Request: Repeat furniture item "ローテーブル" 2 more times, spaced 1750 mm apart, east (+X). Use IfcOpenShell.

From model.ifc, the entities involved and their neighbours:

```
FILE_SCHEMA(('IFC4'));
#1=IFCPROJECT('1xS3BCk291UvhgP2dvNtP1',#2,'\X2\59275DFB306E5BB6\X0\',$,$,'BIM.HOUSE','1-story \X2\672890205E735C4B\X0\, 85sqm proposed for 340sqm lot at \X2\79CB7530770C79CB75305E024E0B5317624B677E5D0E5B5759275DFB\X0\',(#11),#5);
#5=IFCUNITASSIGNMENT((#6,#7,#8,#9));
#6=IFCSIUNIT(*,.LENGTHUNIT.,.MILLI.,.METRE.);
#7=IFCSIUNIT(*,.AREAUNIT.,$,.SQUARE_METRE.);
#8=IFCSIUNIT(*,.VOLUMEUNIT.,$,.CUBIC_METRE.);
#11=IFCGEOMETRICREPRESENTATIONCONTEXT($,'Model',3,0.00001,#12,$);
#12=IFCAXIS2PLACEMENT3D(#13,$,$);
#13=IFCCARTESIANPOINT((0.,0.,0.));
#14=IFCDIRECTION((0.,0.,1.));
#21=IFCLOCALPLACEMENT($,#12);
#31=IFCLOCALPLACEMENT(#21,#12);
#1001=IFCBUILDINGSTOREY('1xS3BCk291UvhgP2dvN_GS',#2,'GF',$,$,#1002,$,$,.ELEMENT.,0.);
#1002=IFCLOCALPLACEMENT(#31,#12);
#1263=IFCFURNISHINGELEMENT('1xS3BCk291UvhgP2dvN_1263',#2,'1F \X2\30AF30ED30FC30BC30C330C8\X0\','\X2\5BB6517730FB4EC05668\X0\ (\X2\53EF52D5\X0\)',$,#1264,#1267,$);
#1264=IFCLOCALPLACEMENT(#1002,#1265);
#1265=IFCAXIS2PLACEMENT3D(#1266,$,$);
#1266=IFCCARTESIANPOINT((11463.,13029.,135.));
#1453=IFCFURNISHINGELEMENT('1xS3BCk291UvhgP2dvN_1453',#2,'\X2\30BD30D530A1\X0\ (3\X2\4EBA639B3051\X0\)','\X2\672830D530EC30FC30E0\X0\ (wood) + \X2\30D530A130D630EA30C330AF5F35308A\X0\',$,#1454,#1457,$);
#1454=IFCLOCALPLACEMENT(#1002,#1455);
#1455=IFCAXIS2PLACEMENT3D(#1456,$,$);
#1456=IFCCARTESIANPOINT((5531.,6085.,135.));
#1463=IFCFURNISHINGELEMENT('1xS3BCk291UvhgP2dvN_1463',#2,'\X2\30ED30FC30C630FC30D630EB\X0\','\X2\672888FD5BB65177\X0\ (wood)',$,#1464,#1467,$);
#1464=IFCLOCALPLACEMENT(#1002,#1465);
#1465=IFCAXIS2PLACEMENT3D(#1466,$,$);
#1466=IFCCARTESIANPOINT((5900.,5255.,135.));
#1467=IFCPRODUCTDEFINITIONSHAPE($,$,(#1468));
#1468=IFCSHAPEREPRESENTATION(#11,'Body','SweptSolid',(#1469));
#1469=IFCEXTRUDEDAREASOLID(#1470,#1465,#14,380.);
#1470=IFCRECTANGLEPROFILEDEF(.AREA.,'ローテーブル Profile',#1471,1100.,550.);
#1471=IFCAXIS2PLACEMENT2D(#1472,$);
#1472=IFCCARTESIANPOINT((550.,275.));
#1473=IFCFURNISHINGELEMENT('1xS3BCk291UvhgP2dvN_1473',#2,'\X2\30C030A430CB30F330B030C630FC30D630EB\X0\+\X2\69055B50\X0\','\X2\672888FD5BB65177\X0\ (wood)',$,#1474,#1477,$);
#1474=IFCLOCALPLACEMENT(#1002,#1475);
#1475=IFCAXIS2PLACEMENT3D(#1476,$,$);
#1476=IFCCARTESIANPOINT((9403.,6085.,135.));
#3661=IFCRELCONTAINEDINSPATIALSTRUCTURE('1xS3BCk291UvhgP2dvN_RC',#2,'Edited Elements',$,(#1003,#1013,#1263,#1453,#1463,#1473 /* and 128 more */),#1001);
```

```python
import numpy as np
import ifcopenshell
import ifcopenshell.api.geometry
import ifcopenshell.api.root
import ifcopenshell.util.element
import ifcopenshell.util.placement
import ifcopenshell.util.unit

model = ifcopenshell.open("model.ifc")
unit_scale = ifcopenshell.util.unit.calculate_unit_scale(model)


def reuse_history(source, copy):
    """copy_class also copies each property set's owner history, people and application; keep the originals."""
    for rel in copy.IsDefinedBy:
        if rel.is_a("IfcRelDefinesByProperties") and (history := rel.RelatingPropertyDefinition.OwnerHistory):
            rel.RelatingPropertyDefinition.OwnerHistory = source.OwnerHistory
            ifcopenshell.util.element.remove_deep2(model, history)


source = model.by_guid("1xS3BCk291UvhgP2dvN_1463")
base = ifcopenshell.util.placement.get_local_placement(source.ObjectPlacement)
step = np.array([1.0, 0.0, 0.0]) * 1.75 / unit_scale

for i in range(1, 3):
    copy = ifcopenshell.api.root.copy_class(model, product=source)
    copy.Representation = ifcopenshell.util.element.copy_deep(
        model, source.Representation, exclude=["IfcGeometricRepresentationContext", "IfcRepresentationMap"]
    )
    reuse_history(source, copy)
    matrix = base.copy()
    matrix[:3, 3] += i * step
    print("added at", matrix[:3, 3].round(3) + 0.0)
    ifcopenshell.api.geometry.edit_object_placement(model, product=copy, matrix=matrix, is_si=False)

model.write("model_updated.ifc")
```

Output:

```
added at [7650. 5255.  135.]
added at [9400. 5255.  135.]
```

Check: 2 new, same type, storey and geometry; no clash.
